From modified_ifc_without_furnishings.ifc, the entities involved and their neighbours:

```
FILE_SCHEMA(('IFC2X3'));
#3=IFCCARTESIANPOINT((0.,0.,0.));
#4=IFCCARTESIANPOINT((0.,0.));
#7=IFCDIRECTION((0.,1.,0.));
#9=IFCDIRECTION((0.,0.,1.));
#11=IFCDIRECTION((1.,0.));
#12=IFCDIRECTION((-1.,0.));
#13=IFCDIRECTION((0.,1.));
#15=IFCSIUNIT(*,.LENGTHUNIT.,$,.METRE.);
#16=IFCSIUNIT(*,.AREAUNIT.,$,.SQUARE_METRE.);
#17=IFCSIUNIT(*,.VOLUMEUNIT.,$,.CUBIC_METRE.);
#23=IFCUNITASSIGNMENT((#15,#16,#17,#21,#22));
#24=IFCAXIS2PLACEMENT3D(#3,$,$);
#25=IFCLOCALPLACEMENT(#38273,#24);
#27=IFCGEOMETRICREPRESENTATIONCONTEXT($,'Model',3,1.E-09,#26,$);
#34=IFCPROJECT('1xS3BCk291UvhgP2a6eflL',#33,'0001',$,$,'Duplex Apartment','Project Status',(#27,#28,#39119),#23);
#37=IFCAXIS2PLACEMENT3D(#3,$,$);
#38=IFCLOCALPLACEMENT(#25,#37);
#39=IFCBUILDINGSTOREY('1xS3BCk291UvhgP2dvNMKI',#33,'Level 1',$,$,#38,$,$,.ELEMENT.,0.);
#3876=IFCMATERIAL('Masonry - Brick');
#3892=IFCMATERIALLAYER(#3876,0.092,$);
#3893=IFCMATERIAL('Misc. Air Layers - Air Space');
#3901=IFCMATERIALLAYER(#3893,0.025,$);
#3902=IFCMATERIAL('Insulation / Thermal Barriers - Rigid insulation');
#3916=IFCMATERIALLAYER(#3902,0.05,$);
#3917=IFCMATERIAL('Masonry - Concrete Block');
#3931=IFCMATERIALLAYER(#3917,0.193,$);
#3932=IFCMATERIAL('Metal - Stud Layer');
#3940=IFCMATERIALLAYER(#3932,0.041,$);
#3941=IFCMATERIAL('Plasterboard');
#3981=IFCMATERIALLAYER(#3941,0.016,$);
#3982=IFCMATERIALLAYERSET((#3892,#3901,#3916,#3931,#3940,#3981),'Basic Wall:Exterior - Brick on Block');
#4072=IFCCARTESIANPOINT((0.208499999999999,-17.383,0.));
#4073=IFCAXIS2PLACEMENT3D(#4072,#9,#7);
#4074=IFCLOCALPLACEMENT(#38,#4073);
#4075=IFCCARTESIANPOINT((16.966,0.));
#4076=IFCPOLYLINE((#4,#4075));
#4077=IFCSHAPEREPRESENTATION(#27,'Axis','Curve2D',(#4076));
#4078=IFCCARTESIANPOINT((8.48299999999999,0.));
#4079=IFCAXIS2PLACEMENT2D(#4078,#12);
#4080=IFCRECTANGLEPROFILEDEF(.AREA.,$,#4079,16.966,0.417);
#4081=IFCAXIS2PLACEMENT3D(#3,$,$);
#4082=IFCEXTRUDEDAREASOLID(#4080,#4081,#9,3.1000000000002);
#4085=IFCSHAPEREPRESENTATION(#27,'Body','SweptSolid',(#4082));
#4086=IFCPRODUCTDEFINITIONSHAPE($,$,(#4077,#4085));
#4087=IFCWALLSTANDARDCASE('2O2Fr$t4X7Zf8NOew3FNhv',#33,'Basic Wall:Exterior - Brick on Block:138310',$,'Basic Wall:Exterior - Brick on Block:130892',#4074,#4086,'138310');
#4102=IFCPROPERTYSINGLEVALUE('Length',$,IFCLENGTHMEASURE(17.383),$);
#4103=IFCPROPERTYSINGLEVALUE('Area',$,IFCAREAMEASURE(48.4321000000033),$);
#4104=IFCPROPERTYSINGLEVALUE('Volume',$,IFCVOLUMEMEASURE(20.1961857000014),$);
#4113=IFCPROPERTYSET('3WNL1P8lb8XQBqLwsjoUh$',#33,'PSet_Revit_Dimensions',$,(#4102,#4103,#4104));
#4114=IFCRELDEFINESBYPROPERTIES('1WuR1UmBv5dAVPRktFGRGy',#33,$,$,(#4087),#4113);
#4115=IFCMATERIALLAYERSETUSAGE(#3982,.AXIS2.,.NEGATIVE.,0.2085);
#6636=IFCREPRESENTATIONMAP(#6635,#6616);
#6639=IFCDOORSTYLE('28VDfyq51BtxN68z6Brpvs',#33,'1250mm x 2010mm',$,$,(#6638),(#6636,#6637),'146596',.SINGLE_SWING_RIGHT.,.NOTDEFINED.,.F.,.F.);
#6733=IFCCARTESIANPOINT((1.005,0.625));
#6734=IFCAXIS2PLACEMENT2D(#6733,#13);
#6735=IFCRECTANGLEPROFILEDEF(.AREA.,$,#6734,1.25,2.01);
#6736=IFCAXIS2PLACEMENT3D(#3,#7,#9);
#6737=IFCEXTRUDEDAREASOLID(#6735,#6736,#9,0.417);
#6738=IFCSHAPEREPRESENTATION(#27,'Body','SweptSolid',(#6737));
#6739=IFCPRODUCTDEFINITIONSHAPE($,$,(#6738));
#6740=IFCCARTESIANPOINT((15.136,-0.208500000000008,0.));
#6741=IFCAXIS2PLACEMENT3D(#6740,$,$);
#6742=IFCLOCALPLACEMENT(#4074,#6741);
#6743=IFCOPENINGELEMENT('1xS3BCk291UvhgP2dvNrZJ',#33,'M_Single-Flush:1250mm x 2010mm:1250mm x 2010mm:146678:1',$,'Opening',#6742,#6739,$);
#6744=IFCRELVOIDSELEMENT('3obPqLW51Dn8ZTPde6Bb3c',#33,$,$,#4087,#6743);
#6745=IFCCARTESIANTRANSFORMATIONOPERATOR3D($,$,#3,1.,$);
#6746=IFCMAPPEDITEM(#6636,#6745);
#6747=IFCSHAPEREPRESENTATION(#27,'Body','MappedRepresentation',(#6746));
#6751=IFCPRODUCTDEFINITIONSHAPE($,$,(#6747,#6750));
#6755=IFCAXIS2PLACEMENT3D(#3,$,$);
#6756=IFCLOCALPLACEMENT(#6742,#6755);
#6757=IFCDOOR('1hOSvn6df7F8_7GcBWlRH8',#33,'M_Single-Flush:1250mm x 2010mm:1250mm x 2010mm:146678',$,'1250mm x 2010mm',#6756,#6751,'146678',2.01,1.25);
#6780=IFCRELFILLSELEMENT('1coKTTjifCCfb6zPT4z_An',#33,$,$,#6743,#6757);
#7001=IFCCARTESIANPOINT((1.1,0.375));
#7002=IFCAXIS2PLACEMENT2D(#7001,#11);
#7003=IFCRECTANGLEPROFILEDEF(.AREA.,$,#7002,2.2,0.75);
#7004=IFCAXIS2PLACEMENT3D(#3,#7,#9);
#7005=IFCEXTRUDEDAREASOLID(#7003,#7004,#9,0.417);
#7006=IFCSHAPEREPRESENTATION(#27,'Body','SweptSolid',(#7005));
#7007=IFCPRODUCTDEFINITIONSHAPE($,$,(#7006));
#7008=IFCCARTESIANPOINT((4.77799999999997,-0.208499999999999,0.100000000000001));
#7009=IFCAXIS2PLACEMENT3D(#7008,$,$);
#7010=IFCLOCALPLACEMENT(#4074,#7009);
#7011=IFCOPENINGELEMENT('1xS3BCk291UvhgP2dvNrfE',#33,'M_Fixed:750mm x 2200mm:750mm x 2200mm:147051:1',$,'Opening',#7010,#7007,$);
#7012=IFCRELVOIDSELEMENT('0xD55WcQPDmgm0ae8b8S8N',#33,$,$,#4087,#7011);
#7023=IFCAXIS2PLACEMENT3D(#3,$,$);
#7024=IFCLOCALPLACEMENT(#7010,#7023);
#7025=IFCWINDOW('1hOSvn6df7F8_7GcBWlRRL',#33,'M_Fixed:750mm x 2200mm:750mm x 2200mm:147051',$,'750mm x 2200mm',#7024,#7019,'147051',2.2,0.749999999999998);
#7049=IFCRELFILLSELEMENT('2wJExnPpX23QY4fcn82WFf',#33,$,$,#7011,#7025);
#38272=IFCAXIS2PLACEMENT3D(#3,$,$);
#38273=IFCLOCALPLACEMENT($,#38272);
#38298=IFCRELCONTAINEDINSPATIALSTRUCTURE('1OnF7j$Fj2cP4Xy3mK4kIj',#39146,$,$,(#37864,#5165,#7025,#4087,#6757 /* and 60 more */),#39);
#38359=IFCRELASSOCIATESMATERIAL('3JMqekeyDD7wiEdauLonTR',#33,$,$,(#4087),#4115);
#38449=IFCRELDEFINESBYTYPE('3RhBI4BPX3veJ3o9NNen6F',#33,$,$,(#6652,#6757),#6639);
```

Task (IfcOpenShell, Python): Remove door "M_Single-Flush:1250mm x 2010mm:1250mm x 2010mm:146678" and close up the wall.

```python
import ifcopenshell
import ifcopenshell.api.feature
import ifcopenshell.api.pset
import ifcopenshell.api.root
import ifcopenshell.geom
import ifcopenshell.util.element
import ifcopenshell.util.shape
import ifcopenshell.util.unit

model = ifcopenshell.open("modified_ifc_without_furnishings.ifc")
area_scale = ifcopenshell.util.unit.calculate_unit_scale(model, "AREAUNIT")
volume_scale = ifcopenshell.util.unit.calculate_unit_scale(model, "VOLUMEUNIT")
settings = ifcopenshell.geom.settings()


def volume(element):
    """Net volume in cubic metres, openings subtracted."""
    shape = ifcopenshell.geom.create_shape(settings, element)
    return ifcopenshell.util.shape.get_volume(shape.geometry)


door = model.by_id(6757)
opening = door.FillsVoids[0].RelatingOpeningElement
wall = opening.VoidsElements[0].RelatingBuildingElement
before = volume(wall)

ifcopenshell.api.root.remove_product(model, product=door)
ifcopenshell.api.feature.remove_feature(model, feature=opening)

after = volume(wall)
thickness = 0.417  # wall thickness in metres

# Update the wall's stored quantities.
pset = model.by_id(ifcopenshell.util.element.get_pset(wall, "PSet_Revit_Dimensions", should_inherit=False)["id"])
ifcopenshell.api.pset.edit_pset(model, pset=pset, properties={
    "Area": model.create_entity("IfcAreaMeasure", after / thickness / area_scale),
    "Volume": model.create_entity("IfcVolumeMeasure", after / volume_scale),
})

print(f"wall volume {before:.3f} -> {after:.3f} m3")

model.write("modified_ifc_without_furnishings_rev.ifc")
```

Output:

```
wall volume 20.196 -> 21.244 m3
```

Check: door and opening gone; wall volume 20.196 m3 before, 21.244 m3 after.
